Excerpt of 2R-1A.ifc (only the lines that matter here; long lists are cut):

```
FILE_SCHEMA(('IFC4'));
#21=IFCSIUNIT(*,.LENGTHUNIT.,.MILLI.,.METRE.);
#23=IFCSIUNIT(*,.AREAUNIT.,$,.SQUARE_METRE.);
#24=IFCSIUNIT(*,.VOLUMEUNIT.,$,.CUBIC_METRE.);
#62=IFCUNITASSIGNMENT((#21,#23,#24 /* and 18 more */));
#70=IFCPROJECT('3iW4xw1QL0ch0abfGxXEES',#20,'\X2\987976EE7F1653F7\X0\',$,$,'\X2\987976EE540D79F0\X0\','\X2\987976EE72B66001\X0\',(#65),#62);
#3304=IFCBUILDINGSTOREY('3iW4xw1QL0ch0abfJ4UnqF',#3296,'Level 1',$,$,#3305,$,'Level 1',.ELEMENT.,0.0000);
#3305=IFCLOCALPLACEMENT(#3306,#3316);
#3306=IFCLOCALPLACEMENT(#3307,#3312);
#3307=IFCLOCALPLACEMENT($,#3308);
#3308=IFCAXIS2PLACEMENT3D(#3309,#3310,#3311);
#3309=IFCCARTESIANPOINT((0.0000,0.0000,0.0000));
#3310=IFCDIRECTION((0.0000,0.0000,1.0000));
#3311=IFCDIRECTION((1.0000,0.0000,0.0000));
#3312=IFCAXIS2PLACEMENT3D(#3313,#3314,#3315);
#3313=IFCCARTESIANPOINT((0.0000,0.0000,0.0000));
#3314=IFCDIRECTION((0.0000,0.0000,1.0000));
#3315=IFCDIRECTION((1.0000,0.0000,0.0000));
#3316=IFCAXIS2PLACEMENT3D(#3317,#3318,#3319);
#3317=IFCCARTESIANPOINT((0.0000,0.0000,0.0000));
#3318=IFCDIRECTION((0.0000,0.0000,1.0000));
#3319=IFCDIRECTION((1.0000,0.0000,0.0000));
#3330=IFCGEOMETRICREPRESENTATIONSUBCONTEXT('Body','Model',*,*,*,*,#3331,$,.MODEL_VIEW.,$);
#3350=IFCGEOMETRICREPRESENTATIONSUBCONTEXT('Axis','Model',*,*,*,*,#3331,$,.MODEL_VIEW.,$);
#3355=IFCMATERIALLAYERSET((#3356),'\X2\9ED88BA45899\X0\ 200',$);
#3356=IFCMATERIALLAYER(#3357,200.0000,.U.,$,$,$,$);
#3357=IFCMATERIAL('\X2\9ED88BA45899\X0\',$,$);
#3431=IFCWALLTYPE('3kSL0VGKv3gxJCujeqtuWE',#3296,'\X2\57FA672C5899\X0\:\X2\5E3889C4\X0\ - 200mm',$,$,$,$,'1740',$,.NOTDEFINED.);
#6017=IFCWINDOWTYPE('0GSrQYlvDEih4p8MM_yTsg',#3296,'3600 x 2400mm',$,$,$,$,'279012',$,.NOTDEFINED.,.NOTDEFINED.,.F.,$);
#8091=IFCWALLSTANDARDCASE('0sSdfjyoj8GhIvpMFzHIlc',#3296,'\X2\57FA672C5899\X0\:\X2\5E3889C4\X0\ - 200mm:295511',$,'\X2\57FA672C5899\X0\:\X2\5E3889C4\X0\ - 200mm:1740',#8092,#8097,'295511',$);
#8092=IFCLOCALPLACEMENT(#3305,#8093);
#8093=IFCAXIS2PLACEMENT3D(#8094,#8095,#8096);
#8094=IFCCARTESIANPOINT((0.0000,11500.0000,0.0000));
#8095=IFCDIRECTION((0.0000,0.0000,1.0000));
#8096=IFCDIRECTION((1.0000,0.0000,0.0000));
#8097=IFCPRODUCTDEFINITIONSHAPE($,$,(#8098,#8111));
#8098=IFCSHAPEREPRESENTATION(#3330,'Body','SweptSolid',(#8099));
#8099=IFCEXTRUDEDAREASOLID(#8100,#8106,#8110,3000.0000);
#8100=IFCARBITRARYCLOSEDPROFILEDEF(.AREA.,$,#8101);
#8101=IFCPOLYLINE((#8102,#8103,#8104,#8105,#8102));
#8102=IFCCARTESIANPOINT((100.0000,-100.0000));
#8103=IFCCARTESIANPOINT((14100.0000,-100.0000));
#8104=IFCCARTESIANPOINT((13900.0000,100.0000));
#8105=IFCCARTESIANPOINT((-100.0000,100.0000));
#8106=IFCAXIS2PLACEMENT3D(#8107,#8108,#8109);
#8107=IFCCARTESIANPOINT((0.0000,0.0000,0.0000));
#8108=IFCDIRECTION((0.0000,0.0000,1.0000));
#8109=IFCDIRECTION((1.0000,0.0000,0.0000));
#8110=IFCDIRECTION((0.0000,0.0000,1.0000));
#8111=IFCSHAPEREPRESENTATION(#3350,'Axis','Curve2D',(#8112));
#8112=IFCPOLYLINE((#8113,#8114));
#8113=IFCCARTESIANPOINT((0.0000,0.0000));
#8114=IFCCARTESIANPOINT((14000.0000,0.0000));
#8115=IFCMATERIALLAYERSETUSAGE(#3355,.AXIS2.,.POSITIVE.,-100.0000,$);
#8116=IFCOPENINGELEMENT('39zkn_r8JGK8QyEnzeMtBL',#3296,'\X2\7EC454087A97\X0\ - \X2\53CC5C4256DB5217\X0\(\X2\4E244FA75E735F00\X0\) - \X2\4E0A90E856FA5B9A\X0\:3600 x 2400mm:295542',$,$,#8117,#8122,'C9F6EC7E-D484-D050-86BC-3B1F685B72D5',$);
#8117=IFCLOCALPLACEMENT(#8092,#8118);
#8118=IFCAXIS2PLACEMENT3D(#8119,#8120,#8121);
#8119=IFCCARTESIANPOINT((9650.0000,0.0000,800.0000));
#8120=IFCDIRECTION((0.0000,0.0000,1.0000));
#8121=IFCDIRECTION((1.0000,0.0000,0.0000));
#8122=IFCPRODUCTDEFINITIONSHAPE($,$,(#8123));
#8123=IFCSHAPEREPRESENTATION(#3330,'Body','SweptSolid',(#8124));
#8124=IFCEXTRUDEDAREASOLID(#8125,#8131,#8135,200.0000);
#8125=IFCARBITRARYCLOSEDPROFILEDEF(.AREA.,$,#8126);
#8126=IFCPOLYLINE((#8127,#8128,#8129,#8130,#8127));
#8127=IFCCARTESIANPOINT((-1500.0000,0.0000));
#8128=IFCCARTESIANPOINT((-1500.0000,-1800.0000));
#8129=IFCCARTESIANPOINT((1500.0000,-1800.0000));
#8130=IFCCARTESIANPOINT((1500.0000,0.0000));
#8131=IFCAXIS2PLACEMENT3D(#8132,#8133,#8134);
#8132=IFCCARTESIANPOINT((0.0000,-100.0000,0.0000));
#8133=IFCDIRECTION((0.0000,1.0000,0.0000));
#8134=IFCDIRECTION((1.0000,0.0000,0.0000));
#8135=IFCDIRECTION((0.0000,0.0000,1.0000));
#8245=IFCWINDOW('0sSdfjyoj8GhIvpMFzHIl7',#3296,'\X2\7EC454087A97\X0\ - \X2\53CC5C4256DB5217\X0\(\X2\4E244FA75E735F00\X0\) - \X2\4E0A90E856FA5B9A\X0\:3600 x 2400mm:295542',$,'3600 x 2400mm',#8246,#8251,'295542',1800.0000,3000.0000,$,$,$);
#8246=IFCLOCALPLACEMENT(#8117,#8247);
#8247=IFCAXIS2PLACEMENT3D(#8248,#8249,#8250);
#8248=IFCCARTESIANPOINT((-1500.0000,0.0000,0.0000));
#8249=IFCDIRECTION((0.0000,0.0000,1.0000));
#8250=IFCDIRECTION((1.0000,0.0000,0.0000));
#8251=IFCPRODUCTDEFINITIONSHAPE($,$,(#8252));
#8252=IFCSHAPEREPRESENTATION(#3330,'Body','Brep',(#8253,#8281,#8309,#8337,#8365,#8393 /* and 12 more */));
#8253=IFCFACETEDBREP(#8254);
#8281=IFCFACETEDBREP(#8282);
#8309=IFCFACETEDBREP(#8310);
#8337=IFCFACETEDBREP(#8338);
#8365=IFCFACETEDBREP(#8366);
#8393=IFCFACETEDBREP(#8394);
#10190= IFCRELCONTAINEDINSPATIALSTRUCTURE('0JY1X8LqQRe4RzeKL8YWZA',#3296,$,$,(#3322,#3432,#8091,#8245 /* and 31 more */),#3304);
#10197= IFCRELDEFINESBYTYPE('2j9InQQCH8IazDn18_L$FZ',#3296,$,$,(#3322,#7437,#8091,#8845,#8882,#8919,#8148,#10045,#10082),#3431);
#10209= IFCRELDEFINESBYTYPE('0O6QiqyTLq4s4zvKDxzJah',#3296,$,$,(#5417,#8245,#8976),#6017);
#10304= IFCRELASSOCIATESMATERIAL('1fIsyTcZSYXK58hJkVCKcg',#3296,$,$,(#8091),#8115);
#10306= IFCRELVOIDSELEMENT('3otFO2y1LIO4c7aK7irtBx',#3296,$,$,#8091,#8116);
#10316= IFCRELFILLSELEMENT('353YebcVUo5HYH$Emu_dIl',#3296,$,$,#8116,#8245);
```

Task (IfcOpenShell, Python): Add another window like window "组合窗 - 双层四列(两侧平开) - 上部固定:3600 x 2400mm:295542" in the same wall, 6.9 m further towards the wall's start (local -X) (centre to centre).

```python
import ifcopenshell
import ifcopenshell.api.feature
import ifcopenshell.api.geometry
import ifcopenshell.api.root
import ifcopenshell.geom
import ifcopenshell.util.element
import ifcopenshell.util.placement
import ifcopenshell.util.shape

model = ifcopenshell.open("2R-1A.ifc")
settings = ifcopenshell.geom.settings()


def volume(element):
    """Net volume in cubic metres, openings subtracted."""
    shape = ifcopenshell.geom.create_shape(settings, element)
    return ifcopenshell.util.shape.get_volume(shape.geometry)


def reuse_history(source, copy):
    """copy_class also copies each property set's owner history, people and application; keep the originals."""
    for rel in copy.IsDefinedBy:
        if rel.is_a("IfcRelDefinesByProperties") and (history := rel.RelatingPropertyDefinition.OwnerHistory):
            rel.RelatingPropertyDefinition.OwnerHistory = source.OwnerHistory
            ifcopenshell.util.element.remove_deep2(model, history)


window = model.by_guid("0sSdfjyoj8GhIvpMFzHIl7")
opening = window.FillsVoids[0].RelatingOpeningElement
wall = opening.VoidsElements[0].RelatingBuildingElement
before = volume(wall)
shift = ifcopenshell.util.placement.get_local_placement(wall.ObjectPlacement)[:3, 0] * -6900.0

# copy_class copies the void relationship, type, container and properties, but no geometry.
new_opening = ifcopenshell.api.root.copy_class(model, product=opening)
new_opening.Representation = ifcopenshell.util.element.copy_deep(
    model, opening.Representation, exclude=["IfcGeometricRepresentationContext", "IfcRepresentationMap"]
)
new_opening.Name = "组合窗 - 双层四列(两侧平开) - 上部固定:3600 x 2400mm"
new_opening.Tag = None
new_window = ifcopenshell.api.root.copy_class(model, product=window)
new_window.Representation = ifcopenshell.util.element.copy_deep(
    model, window.Representation, exclude=["IfcGeometricRepresentationContext", "IfcRepresentationMap"]
)
new_window.Name = "组合窗 - 双层四列(两侧平开) - 上部固定:3600 x 2400mm"
new_window.Tag = None
reuse_history(window, new_window)
ifcopenshell.api.feature.add_filling(model, opening=new_opening, element=new_window)

for old, new in ((opening, new_opening), (window, new_window)):
    matrix = ifcopenshell.util.placement.get_local_placement(old.ObjectPlacement)
    matrix[:3, 3] += shift
    ifcopenshell.api.geometry.edit_object_placement(model, product=new, matrix=matrix, is_si=False)

after = volume(wall)

print(f"wall volume {before:.3f} -> {after:.3f} m3")

model.write("2R-1A_rev.ifc")
```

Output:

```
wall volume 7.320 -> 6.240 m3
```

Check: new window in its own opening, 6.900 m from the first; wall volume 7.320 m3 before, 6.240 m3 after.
